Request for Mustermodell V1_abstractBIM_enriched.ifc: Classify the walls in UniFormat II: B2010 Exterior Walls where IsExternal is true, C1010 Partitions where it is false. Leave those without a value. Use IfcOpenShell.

First a look at what the model holds.

```python
import ifcopenshell
import ifcopenshell.util.element

model = ifcopenshell.open("Mustermodell V1_abstractBIM_enriched.ifc")
print(model.schema)
print("classifications:", [c.Name for c in model.by_type("IfcClassification")])
values = [ifcopenshell.util.element.get_pset(e, "Pset_WallCommon", "IsExternal") for e in model.by_type("IfcWall")]
for value in (True, False, None):
    print("IsExternal", value, values.count(value))
```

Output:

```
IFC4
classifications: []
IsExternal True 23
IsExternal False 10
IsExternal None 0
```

```python
import ifcopenshell
import ifcopenshell.api.classification
import ifcopenshell.util.element

model = ifcopenshell.open("Mustermodell V1_abstractBIM_enriched.ifc")

system = ifcopenshell.api.classification.add_classification(model, classification="UniFormat II")

walls = model.by_type("IfcWall")
external = {e: ifcopenshell.util.element.get_pset(e, "Pset_WallCommon", "IsExternal") for e in walls}
for flag, code, name in ((True, "B2010", "Exterior Walls"), (False, "C1010", "Partitions")):
    products = [e for e in walls if external[e] is flag]
    ifcopenshell.api.classification.add_reference(
        model, products=products, classification=system, identification=code, name=name
    )
    print(code, len(products))

model.write("Mustermodell V1_abstractBIM_enriched-out.ifc")
```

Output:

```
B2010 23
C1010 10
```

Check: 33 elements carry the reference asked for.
